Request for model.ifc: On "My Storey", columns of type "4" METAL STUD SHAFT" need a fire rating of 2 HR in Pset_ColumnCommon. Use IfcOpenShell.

First a look at what the model holds.

```python
import ifcopenshell
import ifcopenshell.util.element

model = ifcopenshell.open("model.ifc")
print(model.schema)
storey = next(s for s in model.by_type("IfcBuildingStorey") if s.Name == "My Storey")
columns = [e for e in ifcopenshell.util.element.get_decomposition(storey) if e.is_a("IfcColumn")]
seen = {}
for e in columns:
    element_type = ifcopenshell.util.element.get_type(e)
    key = (element_type.Name if element_type != e and element_type else None, ifcopenshell.util.element.get_pset(e, "Pset_ColumnCommon", "FireRating"))
    seen[key] = seen.get(key, 0) + 1
for (name, value), count in sorted(seen.items(), key=str):
    print(count, "x", name, "|", value)
```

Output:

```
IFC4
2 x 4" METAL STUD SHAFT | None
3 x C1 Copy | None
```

```python
import ifcopenshell
import ifcopenshell.api.pset
import ifcopenshell.util.element

model = ifcopenshell.open("model.ifc")

storey = next(s for s in model.by_type("IfcBuildingStorey") if s.Name == "My Storey")
columns = [e for e in ifcopenshell.util.element.get_decomposition(storey) if e.is_a("IfcColumn")]

count = 0
for e in columns:
    element_type = ifcopenshell.util.element.get_type(e)
    if element_type in (None, e) or element_type.Name != '4" METAL STUD SHAFT':
        continue
    # add_pset returns the element's existing set when there is one.
    pset = ifcopenshell.api.pset.add_pset(model, product=e, name="Pset_ColumnCommon")
    ifcopenshell.api.pset.edit_pset(model, pset=pset, properties={"FireRating": "2 HR"})
    count += 1

print(count, "columns updated")

model.write("model_v2.ifc")
```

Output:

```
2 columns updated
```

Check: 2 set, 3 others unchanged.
